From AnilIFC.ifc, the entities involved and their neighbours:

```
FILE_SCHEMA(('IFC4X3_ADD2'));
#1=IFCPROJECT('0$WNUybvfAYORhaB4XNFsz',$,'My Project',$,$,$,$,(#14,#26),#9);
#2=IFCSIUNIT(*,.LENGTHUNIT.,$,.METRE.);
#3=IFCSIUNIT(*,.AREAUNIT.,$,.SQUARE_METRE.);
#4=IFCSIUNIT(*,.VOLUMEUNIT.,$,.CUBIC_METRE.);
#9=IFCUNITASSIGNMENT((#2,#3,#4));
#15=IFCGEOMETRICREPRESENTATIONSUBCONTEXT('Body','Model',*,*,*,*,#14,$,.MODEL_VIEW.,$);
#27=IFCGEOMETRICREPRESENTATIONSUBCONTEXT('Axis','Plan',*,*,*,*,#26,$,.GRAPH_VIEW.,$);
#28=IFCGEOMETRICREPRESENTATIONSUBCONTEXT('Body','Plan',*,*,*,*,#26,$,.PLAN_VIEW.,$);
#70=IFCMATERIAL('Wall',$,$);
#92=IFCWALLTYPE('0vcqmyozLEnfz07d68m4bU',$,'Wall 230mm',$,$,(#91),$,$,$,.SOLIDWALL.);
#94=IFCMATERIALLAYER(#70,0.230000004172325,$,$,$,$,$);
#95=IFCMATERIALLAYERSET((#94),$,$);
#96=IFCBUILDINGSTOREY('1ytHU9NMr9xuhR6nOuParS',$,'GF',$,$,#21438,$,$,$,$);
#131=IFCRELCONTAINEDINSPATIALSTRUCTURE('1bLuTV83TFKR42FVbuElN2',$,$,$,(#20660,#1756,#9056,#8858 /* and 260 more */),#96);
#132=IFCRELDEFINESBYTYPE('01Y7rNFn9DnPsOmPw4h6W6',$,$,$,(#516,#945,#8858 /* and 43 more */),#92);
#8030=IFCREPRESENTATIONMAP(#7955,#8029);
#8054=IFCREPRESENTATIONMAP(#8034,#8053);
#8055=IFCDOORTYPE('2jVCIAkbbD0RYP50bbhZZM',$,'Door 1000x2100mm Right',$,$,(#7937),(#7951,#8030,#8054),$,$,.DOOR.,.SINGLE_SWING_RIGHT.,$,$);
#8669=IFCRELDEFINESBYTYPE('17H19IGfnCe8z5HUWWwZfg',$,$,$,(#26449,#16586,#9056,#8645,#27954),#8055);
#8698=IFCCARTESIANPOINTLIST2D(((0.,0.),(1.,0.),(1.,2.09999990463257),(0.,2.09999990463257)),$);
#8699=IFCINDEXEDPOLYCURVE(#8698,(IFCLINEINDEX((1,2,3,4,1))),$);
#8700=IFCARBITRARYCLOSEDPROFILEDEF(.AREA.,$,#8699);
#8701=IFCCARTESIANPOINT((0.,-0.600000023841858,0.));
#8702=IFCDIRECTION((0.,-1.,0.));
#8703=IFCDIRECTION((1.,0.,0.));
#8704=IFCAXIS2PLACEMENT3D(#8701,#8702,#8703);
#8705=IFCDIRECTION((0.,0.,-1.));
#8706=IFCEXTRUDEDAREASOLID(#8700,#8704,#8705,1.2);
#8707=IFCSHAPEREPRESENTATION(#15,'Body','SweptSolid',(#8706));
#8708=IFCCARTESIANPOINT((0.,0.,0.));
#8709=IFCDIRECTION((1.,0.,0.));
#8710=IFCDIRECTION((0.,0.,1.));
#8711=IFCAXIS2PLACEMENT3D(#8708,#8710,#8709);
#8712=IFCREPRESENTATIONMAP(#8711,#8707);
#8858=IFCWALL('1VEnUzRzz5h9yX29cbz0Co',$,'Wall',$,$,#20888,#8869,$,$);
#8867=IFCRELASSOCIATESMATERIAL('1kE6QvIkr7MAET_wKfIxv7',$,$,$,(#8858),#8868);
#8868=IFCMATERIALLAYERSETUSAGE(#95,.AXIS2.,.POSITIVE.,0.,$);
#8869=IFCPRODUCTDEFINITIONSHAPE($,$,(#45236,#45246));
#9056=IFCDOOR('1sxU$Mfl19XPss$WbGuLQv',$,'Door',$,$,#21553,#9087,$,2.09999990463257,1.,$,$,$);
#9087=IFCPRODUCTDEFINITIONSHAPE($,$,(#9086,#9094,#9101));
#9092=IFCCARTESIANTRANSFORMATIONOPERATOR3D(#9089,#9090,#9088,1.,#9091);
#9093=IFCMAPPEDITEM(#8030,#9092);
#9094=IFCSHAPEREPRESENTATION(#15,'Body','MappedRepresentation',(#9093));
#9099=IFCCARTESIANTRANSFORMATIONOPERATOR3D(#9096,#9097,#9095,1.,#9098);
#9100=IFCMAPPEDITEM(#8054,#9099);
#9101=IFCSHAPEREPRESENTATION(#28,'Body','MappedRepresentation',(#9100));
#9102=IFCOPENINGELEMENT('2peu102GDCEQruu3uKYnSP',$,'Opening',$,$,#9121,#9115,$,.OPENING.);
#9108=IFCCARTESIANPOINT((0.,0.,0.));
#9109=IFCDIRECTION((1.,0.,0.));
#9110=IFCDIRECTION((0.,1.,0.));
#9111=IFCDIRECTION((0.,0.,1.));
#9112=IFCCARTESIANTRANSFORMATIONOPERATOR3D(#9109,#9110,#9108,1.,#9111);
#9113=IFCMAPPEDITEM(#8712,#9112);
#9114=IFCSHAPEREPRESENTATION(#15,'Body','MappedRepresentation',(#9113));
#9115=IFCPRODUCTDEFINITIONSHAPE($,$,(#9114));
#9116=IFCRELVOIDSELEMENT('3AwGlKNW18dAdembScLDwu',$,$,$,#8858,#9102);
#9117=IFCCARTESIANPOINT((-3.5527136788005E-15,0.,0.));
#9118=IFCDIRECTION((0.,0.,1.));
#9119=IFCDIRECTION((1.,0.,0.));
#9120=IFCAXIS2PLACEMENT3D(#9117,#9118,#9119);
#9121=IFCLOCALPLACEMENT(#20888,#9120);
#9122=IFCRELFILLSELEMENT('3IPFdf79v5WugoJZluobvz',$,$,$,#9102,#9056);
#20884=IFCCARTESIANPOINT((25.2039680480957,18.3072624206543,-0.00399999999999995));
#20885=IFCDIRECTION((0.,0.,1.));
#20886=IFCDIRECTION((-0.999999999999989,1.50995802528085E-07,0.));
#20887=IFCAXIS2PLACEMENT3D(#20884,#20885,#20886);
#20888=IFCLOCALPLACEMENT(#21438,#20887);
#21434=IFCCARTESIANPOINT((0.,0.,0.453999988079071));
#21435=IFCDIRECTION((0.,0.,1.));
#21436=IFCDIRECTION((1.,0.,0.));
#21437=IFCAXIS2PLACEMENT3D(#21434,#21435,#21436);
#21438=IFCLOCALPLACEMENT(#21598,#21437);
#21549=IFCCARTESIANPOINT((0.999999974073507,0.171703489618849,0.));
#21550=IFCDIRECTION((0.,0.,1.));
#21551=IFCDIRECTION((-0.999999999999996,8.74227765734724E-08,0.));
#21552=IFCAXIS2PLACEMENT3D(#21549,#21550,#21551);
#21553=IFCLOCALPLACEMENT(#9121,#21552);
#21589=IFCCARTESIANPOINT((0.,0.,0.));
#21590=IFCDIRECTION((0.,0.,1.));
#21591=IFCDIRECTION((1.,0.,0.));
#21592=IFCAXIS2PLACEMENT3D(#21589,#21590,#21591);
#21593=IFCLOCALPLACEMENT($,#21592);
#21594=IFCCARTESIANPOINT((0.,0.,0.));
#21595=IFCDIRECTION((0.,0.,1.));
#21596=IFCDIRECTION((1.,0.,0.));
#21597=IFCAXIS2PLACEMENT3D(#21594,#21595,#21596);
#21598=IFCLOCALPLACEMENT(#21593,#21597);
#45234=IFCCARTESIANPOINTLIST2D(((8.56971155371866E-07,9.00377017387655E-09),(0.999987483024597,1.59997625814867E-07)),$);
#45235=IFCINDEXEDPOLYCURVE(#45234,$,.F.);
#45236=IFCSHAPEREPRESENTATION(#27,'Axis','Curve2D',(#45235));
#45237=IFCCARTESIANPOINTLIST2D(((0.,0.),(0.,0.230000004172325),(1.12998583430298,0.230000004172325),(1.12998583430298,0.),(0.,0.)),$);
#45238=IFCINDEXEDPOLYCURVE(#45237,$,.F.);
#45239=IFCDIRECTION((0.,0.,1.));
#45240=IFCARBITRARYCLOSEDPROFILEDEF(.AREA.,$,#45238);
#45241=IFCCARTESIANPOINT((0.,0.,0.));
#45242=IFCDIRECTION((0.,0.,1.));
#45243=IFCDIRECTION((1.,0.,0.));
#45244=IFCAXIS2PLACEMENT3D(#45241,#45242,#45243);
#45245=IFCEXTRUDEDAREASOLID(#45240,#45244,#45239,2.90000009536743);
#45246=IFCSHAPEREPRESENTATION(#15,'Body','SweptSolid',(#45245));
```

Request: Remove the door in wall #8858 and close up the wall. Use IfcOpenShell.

```python
import ifcopenshell
import ifcopenshell.api.feature
import ifcopenshell.api.root
import ifcopenshell.geom
import ifcopenshell.util.shape

model = ifcopenshell.open("AnilIFC.ifc")
settings = ifcopenshell.geom.settings()


def volume(element):
    """Net volume in cubic metres, openings subtracted."""
    shape = ifcopenshell.geom.create_shape(settings, element)
    return ifcopenshell.util.shape.get_volume(shape.geometry)


door = model.by_id(9056)
opening = door.FillsVoids[0].RelatingOpeningElement
wall = opening.VoidsElements[0].RelatingBuildingElement
before = volume(wall)

ifcopenshell.api.root.remove_product(model, product=door)
ifcopenshell.api.feature.remove_feature(model, feature=opening)

after = volume(wall)

print(f"wall volume {before:.3f} -> {after:.3f} m3")

model.write("AnilIFC_edited.ifc")
```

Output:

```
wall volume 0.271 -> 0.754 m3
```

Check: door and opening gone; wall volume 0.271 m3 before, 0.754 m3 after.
